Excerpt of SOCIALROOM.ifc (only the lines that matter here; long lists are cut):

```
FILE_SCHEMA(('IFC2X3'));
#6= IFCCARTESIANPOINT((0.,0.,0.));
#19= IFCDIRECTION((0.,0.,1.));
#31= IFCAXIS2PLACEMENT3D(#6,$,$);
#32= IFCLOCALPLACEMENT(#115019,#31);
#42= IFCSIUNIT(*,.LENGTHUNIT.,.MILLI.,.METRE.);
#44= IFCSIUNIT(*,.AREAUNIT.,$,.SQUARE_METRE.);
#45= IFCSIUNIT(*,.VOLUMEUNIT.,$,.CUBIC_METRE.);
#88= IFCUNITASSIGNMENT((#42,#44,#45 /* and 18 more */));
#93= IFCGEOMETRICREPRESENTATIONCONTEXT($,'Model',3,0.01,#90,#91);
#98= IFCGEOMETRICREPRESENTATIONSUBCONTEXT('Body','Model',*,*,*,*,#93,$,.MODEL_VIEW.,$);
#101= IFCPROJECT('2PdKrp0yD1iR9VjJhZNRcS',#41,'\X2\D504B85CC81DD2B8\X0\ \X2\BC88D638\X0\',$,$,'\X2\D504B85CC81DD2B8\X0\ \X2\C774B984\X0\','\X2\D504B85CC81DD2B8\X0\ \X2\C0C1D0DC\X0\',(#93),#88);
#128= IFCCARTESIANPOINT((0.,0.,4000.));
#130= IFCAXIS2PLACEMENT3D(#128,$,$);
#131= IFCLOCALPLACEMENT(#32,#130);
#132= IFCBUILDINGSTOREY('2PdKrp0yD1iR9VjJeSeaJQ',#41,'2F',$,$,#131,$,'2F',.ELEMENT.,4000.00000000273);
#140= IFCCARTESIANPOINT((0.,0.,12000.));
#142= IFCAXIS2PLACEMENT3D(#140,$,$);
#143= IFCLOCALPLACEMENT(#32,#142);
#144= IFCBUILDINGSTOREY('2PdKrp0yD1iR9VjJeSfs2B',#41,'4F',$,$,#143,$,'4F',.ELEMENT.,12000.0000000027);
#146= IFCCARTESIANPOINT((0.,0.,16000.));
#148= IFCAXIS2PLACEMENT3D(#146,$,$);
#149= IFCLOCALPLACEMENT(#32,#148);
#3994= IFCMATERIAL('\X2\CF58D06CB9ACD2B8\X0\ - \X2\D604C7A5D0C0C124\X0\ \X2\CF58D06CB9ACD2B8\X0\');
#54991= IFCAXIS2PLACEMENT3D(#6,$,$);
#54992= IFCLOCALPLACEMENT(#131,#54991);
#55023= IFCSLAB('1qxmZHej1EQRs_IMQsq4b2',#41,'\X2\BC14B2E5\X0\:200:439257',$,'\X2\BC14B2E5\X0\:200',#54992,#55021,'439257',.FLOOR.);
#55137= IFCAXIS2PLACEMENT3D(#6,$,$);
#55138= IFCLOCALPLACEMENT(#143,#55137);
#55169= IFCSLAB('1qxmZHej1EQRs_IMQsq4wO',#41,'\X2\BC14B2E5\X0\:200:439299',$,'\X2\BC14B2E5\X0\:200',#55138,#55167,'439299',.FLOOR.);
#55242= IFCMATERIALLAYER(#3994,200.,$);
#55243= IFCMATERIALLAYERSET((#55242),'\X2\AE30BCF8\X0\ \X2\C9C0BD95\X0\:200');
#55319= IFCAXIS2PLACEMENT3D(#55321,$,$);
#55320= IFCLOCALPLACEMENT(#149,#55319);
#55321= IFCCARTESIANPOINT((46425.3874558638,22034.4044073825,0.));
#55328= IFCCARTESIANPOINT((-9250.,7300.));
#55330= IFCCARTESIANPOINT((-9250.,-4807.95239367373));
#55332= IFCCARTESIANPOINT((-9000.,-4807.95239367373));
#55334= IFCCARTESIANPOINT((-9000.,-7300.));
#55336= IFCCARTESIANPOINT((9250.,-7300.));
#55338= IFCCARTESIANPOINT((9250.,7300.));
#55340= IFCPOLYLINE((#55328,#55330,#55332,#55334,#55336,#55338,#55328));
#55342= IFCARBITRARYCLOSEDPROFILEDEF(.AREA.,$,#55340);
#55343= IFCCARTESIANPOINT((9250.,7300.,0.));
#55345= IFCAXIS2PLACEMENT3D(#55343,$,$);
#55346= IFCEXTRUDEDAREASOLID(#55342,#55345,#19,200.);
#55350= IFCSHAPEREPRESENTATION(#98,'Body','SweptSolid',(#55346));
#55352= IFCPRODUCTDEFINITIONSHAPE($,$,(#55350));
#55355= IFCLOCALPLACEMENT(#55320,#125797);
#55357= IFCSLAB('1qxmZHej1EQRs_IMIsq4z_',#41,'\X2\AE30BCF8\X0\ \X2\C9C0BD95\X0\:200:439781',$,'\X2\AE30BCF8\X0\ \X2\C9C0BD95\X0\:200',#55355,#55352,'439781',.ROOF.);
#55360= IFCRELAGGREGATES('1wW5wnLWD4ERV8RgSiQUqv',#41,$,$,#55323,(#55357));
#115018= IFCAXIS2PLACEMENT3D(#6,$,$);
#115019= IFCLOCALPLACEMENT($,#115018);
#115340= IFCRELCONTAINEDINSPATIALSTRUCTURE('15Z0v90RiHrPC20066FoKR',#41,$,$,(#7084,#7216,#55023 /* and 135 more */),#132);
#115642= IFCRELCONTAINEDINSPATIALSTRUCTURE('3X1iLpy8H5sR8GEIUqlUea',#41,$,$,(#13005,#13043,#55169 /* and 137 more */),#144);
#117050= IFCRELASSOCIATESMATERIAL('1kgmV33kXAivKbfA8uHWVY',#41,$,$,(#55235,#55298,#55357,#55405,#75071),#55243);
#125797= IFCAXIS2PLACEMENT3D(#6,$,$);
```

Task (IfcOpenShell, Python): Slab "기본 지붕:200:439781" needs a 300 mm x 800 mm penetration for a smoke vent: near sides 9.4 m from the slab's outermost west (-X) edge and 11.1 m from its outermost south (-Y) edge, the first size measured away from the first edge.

```python
import numpy as np
import ifcopenshell
import ifcopenshell.api.feature
import ifcopenshell.api.geometry
import ifcopenshell.api.root
import ifcopenshell.geom
import ifcopenshell.util.placement
import ifcopenshell.util.representation
import ifcopenshell.util.shape
import ifcopenshell.util.unit

model = ifcopenshell.open("SOCIALROOM.ifc")
unit_scale = ifcopenshell.util.unit.calculate_unit_scale(model)
settings = ifcopenshell.geom.settings()


def volume(element):
    """Net volume in cubic metres, openings subtracted."""
    shape = ifcopenshell.geom.create_shape(settings, element)
    return ifcopenshell.util.shape.get_volume(shape.geometry)


slab = model.by_guid("1qxmZHej1EQRs_IMIsq4z_")
before = volume(slab)

# Extent in the slab's own axes, in metres. The edges named are its -X and -Y sides.
slab_shape = ifcopenshell.geom.create_shape(settings, slab)
vertices = ifcopenshell.util.shape.get_vertices(slab_shape.geometry)
x_min, y_min, bottom = vertices.min(axis=0)
top = vertices[:, 2].max()

opening = ifcopenshell.api.root.create_entity(model, ifc_class="IfcOpeningElement", name="Smoke vent opening")
context = ifcopenshell.util.representation.get_context(model, "Model", "Body", "MODEL_VIEW")
width, depth = 0.3, 0.8
outline = [(0.0, 0.0), (width, 0.0), (width, depth), (0.0, depth), (0.0, 0.0)]
# Overshoot both faces by 50 mm so the cut is clean.
shape = ifcopenshell.api.geometry.add_slab_representation(
    model, context=context, depth=top - bottom + 0.1, polyline=outline
)
ifcopenshell.api.geometry.assign_representation(model, product=opening, representation=shape)

matrix = ifcopenshell.util.placement.get_local_placement(slab.ObjectPlacement)
matrix[:, 3] = matrix @ np.append(np.array([x_min + 9.4, y_min + 11.1, bottom - 0.05]) / unit_scale, 1.0)
ifcopenshell.api.geometry.edit_object_placement(model, product=opening, matrix=matrix, is_si=False)
ifcopenshell.api.feature.add_feature(model, feature=opening, element=slab)

after = volume(slab)

print(f"slab volume {before:.3f} -> {after:.3f} m3")

model.write("SOCIALROOM_v2.ifc")
```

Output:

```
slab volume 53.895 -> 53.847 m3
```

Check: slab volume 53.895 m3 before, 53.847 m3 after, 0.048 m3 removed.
